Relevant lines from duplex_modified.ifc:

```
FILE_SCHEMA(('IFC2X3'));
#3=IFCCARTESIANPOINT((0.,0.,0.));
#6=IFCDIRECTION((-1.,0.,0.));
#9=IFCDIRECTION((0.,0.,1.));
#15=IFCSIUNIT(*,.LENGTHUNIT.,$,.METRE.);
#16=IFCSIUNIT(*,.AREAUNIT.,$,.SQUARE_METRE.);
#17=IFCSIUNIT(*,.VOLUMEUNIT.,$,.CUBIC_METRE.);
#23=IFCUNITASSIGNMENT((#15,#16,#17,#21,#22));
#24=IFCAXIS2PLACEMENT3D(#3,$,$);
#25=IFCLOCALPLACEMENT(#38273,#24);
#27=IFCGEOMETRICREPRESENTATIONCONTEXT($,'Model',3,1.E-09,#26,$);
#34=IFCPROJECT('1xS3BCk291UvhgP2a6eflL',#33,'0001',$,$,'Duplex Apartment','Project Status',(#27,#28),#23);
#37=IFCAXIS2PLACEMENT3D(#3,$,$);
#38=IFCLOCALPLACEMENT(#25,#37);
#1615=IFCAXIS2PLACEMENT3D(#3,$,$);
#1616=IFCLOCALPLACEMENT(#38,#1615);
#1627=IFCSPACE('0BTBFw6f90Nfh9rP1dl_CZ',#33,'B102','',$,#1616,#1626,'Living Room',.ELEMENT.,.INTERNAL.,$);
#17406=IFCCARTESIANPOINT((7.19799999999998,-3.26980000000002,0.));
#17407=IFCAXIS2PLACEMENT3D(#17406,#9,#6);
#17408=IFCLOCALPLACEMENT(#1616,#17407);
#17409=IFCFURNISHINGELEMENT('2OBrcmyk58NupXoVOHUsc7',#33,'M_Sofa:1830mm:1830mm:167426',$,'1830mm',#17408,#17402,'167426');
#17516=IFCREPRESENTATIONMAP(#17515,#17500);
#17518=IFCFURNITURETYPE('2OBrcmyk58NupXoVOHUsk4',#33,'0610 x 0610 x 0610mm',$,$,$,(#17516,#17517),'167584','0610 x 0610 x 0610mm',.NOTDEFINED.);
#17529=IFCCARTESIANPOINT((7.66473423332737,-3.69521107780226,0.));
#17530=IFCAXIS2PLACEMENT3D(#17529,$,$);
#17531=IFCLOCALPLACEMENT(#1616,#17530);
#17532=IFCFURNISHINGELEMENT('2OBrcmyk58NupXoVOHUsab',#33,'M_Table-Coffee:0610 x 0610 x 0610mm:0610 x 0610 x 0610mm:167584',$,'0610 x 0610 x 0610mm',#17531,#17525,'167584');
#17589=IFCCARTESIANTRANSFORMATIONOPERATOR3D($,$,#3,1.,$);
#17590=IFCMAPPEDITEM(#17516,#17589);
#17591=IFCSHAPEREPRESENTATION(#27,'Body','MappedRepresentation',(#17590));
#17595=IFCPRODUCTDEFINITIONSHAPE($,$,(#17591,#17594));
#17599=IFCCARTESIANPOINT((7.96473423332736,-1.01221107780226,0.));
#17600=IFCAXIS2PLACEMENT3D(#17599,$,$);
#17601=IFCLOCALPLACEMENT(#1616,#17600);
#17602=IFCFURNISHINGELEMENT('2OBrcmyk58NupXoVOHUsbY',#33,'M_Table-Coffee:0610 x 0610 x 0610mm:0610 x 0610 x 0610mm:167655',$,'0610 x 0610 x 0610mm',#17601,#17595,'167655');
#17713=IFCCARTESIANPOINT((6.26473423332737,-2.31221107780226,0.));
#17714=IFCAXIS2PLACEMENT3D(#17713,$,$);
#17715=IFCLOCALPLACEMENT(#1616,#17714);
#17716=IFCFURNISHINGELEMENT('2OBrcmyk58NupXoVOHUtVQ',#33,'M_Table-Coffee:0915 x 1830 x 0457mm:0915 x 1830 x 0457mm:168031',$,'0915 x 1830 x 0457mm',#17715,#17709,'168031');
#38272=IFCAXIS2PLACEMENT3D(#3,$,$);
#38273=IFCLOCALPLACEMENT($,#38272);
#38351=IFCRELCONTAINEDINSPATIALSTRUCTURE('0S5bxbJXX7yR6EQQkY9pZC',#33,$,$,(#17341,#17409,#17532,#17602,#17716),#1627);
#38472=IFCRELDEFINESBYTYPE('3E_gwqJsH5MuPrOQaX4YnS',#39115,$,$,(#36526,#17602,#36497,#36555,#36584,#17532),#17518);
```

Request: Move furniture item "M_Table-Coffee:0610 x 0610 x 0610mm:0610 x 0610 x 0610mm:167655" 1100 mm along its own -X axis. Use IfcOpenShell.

```python
import ifcopenshell
import ifcopenshell.api.geometry
import ifcopenshell.util.placement
import ifcopenshell.util.unit

model = ifcopenshell.open("duplex_modified.ifc")
unit_scale = ifcopenshell.util.unit.calculate_unit_scale(model)

item = model.by_id(17602)
matrix = ifcopenshell.util.placement.get_local_placement(item.ObjectPlacement)
matrix[:3, 3] -= matrix[:3, 0] * 1.1 / unit_scale
ifcopenshell.api.geometry.edit_object_placement(model, product=item, matrix=matrix, is_si=False)

print(ifcopenshell.util.placement.get_local_placement(item.ObjectPlacement).round(3) + 0.0)

model.write("duplex_modified_rev.ifc")
```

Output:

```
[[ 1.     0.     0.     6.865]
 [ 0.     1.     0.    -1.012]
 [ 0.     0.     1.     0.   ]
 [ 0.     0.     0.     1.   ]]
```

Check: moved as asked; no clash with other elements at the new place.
